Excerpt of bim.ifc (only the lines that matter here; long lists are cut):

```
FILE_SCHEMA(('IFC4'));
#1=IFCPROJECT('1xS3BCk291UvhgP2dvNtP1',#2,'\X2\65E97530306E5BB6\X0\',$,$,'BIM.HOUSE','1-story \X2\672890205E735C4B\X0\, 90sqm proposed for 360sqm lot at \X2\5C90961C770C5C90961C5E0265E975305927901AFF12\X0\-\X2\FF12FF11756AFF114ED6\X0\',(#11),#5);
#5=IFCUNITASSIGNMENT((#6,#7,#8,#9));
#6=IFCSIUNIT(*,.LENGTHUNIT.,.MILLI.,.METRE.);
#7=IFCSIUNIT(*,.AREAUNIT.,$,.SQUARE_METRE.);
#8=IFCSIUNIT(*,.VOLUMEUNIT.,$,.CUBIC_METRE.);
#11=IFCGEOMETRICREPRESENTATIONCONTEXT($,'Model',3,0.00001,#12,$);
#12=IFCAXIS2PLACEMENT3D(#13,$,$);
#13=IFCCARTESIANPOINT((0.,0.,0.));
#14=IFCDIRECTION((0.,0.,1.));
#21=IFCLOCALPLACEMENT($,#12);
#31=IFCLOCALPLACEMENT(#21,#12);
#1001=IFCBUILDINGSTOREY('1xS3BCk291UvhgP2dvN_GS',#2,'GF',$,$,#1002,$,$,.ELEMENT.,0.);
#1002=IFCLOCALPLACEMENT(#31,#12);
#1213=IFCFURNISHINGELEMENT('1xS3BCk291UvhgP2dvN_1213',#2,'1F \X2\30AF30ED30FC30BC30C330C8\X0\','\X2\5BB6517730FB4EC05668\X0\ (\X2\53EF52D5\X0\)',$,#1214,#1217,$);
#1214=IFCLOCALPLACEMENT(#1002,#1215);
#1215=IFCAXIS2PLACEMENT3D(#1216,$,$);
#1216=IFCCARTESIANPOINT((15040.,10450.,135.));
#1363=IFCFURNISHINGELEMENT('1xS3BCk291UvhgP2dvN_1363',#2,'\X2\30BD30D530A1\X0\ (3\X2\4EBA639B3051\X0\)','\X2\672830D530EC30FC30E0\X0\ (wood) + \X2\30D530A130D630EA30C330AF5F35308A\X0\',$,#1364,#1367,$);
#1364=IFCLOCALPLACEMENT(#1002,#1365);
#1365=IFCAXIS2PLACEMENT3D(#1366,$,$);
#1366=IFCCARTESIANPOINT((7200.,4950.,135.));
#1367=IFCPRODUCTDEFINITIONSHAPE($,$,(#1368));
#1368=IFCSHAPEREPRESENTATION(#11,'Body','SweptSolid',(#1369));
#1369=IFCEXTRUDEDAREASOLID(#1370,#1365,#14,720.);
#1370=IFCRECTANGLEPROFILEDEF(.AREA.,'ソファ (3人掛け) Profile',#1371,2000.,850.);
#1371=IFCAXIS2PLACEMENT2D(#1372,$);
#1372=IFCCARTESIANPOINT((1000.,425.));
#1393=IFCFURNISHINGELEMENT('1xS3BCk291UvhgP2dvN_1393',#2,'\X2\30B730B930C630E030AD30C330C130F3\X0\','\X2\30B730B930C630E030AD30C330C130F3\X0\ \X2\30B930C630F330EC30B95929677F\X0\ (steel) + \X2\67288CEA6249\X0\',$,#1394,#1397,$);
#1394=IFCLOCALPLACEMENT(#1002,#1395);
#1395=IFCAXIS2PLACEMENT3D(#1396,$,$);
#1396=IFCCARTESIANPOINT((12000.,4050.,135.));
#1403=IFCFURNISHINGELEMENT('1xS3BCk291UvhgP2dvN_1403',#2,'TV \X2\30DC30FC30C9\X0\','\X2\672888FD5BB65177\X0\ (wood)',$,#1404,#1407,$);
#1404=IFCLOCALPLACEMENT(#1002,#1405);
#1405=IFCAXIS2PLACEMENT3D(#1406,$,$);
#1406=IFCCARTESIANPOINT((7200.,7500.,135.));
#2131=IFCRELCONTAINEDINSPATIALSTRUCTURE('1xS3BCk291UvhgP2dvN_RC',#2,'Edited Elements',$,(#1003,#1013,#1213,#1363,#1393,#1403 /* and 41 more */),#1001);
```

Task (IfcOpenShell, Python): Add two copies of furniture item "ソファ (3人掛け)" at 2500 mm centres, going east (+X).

```python
import numpy as np
import ifcopenshell
import ifcopenshell.api.geometry
import ifcopenshell.api.root
import ifcopenshell.util.element
import ifcopenshell.util.placement

model = ifcopenshell.open("bim.ifc")


def reuse_history(source, copy):
    """copy_class also copies each property set's owner history, people and application; keep the originals."""
    for rel in copy.IsDefinedBy:
        if rel.is_a("IfcRelDefinesByProperties") and (history := rel.RelatingPropertyDefinition.OwnerHistory):
            rel.RelatingPropertyDefinition.OwnerHistory = source.OwnerHistory
            ifcopenshell.util.element.remove_deep2(model, history)


source = model.by_guid("1xS3BCk291UvhgP2dvN_1363")
base = ifcopenshell.util.placement.get_local_placement(source.ObjectPlacement)
step = np.array([1.0, 0.0, 0.0]) * 2500.0

for i in range(1, 3):
    copy = ifcopenshell.api.root.copy_class(model, product=source)
    copy.Representation = ifcopenshell.util.element.copy_deep(
        model, source.Representation, exclude=["IfcGeometricRepresentationContext", "IfcRepresentationMap"]
    )
    reuse_history(source, copy)
    matrix = base.copy()
    matrix[:3, 3] += i * step
    print("added at", matrix[:3, 3].round(3) + 0.0)
    ifcopenshell.api.geometry.edit_object_placement(model, product=copy, matrix=matrix, is_si=False)

model.write("bim_edited.ifc")
```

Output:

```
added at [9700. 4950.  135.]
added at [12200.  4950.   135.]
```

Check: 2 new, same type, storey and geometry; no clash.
